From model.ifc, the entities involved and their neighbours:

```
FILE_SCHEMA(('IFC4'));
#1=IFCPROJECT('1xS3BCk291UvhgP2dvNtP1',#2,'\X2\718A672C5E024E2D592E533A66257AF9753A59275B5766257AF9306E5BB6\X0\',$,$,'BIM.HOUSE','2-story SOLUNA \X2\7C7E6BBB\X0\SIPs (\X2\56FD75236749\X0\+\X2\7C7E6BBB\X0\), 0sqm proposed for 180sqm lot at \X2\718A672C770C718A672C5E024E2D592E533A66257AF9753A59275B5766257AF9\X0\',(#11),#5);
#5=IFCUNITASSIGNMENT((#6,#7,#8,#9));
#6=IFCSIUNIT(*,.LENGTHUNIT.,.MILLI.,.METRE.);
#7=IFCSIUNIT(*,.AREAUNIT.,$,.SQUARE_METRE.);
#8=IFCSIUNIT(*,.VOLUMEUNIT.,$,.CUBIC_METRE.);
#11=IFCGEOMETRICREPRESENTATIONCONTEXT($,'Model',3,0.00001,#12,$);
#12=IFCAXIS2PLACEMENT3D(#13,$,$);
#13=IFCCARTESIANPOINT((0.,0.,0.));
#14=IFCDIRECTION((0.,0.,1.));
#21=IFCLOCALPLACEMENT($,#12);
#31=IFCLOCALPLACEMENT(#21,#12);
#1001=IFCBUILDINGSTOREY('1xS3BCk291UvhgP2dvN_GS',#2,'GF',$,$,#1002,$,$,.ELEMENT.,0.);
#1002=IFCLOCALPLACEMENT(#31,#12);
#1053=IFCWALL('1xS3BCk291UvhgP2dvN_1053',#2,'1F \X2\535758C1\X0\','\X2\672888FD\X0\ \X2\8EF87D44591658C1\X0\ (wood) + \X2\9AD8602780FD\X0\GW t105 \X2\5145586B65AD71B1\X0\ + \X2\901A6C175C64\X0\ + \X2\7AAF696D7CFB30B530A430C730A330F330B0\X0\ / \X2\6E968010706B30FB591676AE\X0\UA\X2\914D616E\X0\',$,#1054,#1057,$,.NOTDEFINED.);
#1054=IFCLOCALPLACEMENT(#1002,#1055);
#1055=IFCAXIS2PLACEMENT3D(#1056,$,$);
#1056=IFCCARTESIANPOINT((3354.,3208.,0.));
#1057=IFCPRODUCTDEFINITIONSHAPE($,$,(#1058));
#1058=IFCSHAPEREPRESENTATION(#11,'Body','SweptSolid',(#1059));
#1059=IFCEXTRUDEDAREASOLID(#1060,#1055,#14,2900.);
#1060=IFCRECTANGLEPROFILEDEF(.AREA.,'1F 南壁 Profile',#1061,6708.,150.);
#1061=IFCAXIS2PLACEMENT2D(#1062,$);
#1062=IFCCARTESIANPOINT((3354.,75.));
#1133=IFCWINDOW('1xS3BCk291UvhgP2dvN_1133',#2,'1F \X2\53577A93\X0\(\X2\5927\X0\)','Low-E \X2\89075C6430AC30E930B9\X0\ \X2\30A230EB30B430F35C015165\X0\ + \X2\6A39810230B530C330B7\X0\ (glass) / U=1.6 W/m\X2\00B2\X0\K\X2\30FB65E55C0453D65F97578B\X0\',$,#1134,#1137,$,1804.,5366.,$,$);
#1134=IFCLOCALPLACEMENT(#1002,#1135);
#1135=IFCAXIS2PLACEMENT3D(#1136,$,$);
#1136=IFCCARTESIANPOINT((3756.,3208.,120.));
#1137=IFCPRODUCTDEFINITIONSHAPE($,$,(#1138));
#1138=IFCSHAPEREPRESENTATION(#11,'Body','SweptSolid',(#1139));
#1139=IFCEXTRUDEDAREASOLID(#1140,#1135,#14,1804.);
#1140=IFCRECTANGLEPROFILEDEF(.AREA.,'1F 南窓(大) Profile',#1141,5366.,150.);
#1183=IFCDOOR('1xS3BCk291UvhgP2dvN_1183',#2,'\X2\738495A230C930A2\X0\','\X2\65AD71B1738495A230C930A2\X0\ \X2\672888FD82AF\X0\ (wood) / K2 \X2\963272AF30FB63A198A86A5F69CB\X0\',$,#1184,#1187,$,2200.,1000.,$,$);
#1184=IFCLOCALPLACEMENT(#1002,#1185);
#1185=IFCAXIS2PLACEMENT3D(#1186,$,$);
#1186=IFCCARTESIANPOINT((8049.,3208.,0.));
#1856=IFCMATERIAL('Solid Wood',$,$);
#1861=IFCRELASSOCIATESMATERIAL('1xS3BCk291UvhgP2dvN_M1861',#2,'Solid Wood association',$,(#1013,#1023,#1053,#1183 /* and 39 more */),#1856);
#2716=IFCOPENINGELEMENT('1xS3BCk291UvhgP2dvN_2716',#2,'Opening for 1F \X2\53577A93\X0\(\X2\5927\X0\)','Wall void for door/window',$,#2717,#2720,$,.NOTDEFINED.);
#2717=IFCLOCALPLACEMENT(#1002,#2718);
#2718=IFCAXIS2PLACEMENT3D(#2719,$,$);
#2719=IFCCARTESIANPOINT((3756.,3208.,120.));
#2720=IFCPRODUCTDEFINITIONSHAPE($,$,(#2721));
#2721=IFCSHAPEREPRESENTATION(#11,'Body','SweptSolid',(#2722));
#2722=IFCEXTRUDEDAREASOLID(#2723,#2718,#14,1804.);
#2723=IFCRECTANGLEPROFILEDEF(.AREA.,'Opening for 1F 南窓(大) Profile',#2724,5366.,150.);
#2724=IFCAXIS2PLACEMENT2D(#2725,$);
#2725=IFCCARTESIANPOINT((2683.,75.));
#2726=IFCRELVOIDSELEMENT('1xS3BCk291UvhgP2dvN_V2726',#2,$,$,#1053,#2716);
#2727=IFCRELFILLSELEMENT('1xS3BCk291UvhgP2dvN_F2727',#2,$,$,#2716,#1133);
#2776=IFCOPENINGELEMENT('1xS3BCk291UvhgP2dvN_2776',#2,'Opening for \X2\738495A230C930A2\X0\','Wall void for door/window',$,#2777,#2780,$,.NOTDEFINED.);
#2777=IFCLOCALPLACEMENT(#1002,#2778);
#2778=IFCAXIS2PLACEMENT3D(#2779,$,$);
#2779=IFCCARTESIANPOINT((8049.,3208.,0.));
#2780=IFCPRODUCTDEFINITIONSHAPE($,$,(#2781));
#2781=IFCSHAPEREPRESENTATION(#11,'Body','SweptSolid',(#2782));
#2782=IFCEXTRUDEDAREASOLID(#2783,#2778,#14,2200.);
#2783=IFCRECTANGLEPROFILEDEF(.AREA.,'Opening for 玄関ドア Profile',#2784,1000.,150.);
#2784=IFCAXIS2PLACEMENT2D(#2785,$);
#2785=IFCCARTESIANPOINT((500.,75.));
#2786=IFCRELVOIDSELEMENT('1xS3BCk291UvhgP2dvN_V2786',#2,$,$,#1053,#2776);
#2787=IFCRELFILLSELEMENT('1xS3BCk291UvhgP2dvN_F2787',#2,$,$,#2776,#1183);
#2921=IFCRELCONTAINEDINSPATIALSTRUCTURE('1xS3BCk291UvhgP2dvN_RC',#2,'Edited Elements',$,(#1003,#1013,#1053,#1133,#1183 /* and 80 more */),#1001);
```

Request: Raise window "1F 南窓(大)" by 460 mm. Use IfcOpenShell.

```python
import numpy as np
import ifcopenshell
import ifcopenshell.api.geometry
import ifcopenshell.util.placement
import ifcopenshell.util.unit

model = ifcopenshell.open("model.ifc")
unit_scale = ifcopenshell.util.unit.calculate_unit_scale(model)

window = model.by_guid("1xS3BCk291UvhgP2dvN_1133")
opening = window.FillsVoids[0].RelatingOpeningElement
dz = 460.0

shift = np.array([0.0, 0.0, dz])
# The window is not placed relative to its opening, so move both.
for product in (opening, window):
    matrix = ifcopenshell.util.placement.get_local_placement(product.ObjectPlacement)
    matrix[:3, 3] += shift
    ifcopenshell.api.geometry.edit_object_placement(model, product=product, matrix=matrix, is_si=False)

print(f"moved by {dz * unit_scale:+.3f} m")

model.write("model_updated.ifc")
```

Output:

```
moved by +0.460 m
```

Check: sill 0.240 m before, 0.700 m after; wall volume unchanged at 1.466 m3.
